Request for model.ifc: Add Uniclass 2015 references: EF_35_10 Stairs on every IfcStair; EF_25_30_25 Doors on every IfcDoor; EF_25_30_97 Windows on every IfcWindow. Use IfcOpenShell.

First a look at what the model holds.

```python
import ifcopenshell

model = ifcopenshell.open("model.ifc")
print(model.schema)
print("classifications:", [c.Name for c in model.by_type("IfcClassification")])
for ifc_class in ("IfcDoor", "IfcRoof", "IfcStair", "IfcWall", "IfcWindow"):
    print(ifc_class, len(model.by_type(ifc_class)))
```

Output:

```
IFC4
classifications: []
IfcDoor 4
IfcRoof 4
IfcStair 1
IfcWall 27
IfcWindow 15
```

```python
import ifcopenshell
import ifcopenshell.api.classification

model = ifcopenshell.open("model.ifc")

system = ifcopenshell.api.classification.add_classification(model, classification="Uniclass 2015")

codes = {
    "IfcStair": ("EF_35_10", "Stairs"),
    "IfcDoor": ("EF_25_30_25", "Doors"),
    "IfcWindow": ("EF_25_30_97", "Windows"),
}
for ifc_class, (code, name) in codes.items():
    products = model.by_type(ifc_class)
    ifcopenshell.api.classification.add_reference(
        model, products=products, classification=system, identification=code, name=name
    )
    print(code, len(products))

model.write("model_v2.ifc")
```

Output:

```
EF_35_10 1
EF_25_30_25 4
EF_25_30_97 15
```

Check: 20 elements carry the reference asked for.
